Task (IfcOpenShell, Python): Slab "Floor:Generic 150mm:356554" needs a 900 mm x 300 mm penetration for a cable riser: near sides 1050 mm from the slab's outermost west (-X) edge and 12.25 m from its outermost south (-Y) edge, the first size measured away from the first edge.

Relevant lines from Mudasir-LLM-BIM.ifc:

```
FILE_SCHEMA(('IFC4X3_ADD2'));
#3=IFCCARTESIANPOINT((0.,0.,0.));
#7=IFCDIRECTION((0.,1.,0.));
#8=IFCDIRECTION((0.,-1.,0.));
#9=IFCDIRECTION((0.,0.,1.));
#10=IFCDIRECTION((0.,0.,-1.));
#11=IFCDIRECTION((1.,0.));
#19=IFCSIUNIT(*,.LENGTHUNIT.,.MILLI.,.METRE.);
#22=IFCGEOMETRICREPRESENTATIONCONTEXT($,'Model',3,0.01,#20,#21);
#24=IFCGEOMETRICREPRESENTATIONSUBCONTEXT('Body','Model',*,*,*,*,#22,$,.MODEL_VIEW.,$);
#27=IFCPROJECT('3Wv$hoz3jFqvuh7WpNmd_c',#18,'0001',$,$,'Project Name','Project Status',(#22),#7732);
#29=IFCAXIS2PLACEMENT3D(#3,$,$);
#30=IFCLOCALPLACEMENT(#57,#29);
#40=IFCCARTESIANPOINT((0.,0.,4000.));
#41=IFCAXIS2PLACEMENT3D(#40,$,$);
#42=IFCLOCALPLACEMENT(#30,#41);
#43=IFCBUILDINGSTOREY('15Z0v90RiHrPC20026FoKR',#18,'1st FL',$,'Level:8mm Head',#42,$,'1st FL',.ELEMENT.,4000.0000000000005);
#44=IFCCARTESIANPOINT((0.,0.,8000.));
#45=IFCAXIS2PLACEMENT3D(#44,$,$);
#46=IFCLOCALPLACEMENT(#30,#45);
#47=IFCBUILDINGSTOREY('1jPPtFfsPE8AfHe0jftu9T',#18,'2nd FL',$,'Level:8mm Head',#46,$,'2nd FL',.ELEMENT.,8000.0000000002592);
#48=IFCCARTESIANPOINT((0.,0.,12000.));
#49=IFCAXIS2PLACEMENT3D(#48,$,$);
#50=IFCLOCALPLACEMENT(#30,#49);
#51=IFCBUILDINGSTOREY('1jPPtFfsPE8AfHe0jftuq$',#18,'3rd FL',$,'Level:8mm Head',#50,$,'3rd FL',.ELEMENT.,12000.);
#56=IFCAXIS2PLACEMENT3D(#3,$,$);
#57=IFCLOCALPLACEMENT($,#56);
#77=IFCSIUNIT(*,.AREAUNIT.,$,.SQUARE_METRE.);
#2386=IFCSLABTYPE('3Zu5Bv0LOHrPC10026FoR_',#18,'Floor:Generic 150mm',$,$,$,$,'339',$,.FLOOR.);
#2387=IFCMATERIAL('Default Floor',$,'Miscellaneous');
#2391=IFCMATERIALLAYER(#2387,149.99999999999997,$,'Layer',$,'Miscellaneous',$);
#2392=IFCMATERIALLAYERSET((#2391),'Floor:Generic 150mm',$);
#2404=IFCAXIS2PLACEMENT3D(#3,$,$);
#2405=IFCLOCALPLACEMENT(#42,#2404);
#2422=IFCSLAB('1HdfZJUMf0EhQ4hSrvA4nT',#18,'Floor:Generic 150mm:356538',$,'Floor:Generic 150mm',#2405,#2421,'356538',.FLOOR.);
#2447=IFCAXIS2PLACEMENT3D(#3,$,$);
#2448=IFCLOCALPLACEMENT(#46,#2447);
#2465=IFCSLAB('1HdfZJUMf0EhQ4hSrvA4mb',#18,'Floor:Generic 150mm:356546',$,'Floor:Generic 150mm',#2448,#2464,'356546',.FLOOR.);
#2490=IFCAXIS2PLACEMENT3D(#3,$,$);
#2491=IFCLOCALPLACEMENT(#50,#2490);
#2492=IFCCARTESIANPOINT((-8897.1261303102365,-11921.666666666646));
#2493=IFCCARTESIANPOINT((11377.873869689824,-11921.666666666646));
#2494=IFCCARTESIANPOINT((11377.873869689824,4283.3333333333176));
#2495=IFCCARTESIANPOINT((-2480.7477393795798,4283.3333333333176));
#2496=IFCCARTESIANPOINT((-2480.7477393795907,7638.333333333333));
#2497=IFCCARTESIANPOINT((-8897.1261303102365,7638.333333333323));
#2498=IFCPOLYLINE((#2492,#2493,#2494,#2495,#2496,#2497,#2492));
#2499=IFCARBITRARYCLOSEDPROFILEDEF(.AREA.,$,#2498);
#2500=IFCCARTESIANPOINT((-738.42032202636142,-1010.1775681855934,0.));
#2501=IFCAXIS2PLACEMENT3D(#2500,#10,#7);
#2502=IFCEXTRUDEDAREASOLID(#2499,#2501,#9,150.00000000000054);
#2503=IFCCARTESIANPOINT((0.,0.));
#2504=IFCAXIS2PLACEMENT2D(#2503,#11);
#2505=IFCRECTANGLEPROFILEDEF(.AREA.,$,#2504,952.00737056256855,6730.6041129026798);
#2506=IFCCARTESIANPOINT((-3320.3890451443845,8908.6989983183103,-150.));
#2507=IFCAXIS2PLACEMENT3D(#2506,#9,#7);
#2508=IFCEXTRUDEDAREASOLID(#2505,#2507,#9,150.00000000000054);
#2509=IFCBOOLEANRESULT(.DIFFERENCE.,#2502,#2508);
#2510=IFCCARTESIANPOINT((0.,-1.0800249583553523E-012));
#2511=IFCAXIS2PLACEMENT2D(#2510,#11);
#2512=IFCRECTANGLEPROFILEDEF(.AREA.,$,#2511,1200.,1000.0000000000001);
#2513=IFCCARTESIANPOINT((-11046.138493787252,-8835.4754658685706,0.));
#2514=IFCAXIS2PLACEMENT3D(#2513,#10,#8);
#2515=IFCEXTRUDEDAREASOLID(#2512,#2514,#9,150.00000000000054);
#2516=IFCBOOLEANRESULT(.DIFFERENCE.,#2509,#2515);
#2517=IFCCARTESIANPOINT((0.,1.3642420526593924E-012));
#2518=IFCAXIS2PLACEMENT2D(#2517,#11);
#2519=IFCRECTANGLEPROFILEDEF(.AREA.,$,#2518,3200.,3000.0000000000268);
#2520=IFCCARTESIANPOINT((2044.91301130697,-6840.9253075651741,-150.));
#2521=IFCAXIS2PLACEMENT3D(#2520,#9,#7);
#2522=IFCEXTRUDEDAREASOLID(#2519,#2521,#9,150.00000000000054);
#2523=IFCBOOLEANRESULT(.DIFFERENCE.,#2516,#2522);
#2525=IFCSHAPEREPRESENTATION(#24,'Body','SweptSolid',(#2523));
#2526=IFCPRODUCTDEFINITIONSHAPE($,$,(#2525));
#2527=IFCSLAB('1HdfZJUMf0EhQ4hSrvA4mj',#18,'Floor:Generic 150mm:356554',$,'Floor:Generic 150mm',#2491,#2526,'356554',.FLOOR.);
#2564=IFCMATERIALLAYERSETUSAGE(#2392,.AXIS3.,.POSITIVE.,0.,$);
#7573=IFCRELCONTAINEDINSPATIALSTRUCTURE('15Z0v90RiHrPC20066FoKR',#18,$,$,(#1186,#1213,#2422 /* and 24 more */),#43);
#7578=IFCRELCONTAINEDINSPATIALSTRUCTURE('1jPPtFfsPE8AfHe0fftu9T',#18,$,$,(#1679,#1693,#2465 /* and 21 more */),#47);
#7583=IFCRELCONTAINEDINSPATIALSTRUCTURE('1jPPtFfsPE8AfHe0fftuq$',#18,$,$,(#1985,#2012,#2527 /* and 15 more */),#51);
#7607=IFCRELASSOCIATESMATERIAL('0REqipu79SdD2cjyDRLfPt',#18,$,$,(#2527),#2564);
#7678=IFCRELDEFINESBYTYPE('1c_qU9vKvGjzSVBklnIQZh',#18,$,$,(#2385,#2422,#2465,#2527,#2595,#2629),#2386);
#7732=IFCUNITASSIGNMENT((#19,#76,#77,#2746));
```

```python
import numpy as np
import ifcopenshell
import ifcopenshell.api.feature
import ifcopenshell.api.geometry
import ifcopenshell.api.root
import ifcopenshell.geom
import ifcopenshell.util.placement
import ifcopenshell.util.representation
import ifcopenshell.util.shape
import ifcopenshell.util.unit

model = ifcopenshell.open("Mudasir-LLM-BIM.ifc")
unit_scale = ifcopenshell.util.unit.calculate_unit_scale(model)
settings = ifcopenshell.geom.settings()


def volume(element):
    """Net volume in cubic metres, openings subtracted."""
    shape = ifcopenshell.geom.create_shape(settings, element)
    return ifcopenshell.util.shape.get_volume(shape.geometry)


slab = model.by_guid("1HdfZJUMf0EhQ4hSrvA4mj")
before = volume(slab)

# Extent in the slab's own axes, in metres. The edges named are its -X and -Y sides.
slab_shape = ifcopenshell.geom.create_shape(settings, slab)
vertices = ifcopenshell.util.shape.get_vertices(slab_shape.geometry)
x_min, y_min, bottom = vertices.min(axis=0)
top = vertices[:, 2].max()

opening = ifcopenshell.api.root.create_entity(model, ifc_class="IfcOpeningElement", name="Cable riser opening", predefined_type="OPENING")
context = ifcopenshell.util.representation.get_context(model, "Model", "Body", "MODEL_VIEW")
width, depth = 0.9, 0.3
outline = [(0.0, 0.0), (width, 0.0), (width, depth), (0.0, depth), (0.0, 0.0)]
# Overshoot both faces by 50 mm so the cut is clean.
shape = ifcopenshell.api.geometry.add_slab_representation(
    model, context=context, depth=top - bottom + 0.1, polyline=outline
)
ifcopenshell.api.geometry.assign_representation(model, product=opening, representation=shape)

matrix = ifcopenshell.util.placement.get_local_placement(slab.ObjectPlacement)
matrix[:, 3] = matrix @ np.append(np.array([x_min + 1.05, y_min + 12.25, bottom - 0.05]) / unit_scale, 1.0)
ifcopenshell.api.geometry.edit_object_placement(model, product=opening, matrix=matrix, is_si=False)
ifcopenshell.api.feature.add_feature(model, feature=opening, element=slab)

after = volume(slab)

print(f"slab volume {before:.3f} -> {after:.3f} m3")

model.write("Mudasir-LLM-BIM_edited.ifc")
```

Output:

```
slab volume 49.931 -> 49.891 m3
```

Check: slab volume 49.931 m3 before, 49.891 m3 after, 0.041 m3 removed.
